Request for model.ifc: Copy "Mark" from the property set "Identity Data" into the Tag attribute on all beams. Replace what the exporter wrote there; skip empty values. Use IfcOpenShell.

First a look at what the model holds.

```python
import ifcopenshell
import ifcopenshell.util.element

model = ifcopenshell.open("model.ifc")
print(model.schema)
beams = model.by_type("IfcBeam")
print(len(beams), "beams")
for e in beams[:8]:
    source = ifcopenshell.util.element.get_pset(e, "Identity Data", "Mark")
    target = e.Tag
    print(e.id(), repr(source), repr(target), sep=" | ")
```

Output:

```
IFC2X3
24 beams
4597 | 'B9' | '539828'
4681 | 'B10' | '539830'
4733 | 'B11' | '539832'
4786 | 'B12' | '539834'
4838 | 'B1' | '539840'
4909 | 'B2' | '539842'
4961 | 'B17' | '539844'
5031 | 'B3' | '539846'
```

```python
import ifcopenshell
import ifcopenshell.util.element

model = ifcopenshell.open("model.ifc")

count = 0
for e in model.by_type("IfcBeam"):
    value = ifcopenshell.util.element.get_pset(e, "Identity Data", "Mark")
    current = e.Tag
    if not value or not value.strip() or current == value:
        continue
    e.Tag = value
    count += 1

print(count, "beams updated")

model.write("model_rev.ifc")
```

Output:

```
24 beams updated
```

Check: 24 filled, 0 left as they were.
